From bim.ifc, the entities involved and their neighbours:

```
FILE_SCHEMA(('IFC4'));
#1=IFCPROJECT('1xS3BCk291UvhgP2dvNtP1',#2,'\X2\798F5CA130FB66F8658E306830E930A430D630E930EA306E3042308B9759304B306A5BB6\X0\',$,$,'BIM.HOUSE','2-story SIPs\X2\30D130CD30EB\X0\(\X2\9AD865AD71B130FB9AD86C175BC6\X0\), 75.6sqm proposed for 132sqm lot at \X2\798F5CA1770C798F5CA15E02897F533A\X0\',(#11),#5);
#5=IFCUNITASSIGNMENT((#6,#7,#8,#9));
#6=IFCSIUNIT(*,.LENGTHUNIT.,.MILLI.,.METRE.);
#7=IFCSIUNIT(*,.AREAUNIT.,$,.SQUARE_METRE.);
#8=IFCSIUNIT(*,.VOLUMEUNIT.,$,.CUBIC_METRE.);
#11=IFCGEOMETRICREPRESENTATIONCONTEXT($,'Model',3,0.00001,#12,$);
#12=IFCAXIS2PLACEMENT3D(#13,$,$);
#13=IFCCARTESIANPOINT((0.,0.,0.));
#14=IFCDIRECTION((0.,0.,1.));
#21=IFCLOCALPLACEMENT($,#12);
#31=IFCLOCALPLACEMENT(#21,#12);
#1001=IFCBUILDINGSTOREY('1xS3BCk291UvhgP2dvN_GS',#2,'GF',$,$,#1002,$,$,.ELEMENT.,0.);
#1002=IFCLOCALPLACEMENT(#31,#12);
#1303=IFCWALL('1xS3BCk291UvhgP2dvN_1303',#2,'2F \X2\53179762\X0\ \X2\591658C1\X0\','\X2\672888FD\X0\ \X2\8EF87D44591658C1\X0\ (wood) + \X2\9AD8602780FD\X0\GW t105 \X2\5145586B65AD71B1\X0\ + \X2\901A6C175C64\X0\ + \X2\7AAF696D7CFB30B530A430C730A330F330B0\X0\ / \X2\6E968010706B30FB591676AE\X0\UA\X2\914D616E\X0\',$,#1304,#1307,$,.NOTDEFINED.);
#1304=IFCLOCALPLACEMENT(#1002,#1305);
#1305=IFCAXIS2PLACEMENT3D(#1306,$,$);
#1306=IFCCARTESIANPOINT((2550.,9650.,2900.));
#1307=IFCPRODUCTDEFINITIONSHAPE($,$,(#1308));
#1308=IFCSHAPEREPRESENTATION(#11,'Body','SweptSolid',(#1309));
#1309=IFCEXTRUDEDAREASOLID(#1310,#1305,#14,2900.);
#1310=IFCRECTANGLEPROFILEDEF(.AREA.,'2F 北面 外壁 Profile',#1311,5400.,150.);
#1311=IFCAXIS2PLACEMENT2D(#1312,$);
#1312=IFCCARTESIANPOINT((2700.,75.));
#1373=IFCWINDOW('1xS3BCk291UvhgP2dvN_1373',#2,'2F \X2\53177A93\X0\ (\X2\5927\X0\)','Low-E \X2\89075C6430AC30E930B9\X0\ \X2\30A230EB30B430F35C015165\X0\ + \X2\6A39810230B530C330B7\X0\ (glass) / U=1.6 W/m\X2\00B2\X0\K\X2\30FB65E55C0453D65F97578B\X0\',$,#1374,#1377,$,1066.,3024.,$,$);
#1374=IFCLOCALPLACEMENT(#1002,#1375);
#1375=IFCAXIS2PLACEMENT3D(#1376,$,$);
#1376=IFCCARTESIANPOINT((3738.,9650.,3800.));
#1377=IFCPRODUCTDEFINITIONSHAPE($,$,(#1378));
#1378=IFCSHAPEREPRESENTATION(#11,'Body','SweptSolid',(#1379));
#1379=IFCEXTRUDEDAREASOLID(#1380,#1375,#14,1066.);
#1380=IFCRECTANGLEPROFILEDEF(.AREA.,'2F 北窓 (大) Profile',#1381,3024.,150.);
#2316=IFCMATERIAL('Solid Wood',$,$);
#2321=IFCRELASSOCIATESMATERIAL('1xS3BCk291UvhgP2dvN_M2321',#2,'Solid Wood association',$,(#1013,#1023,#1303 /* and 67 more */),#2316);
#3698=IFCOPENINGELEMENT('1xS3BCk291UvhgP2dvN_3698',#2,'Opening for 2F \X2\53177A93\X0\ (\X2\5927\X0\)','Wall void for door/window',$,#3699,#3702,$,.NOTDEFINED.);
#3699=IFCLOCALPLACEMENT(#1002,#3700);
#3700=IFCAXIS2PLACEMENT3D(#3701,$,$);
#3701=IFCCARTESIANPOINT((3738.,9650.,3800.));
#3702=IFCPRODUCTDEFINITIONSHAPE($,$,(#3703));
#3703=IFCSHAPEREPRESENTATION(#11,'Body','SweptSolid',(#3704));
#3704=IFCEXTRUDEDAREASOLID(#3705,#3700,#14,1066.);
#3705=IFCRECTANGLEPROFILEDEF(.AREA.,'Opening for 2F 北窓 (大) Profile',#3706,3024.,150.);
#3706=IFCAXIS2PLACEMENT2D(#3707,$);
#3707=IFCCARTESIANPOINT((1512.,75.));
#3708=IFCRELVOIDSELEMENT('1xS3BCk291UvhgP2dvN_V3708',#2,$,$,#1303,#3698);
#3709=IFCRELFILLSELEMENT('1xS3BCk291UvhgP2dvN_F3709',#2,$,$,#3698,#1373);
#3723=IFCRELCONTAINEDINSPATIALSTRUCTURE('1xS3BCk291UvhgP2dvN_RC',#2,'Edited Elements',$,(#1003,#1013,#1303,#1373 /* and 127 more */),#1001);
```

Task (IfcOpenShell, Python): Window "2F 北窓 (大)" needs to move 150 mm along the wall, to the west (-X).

```python
import ifcopenshell
import ifcopenshell.api.geometry
import ifcopenshell.util.placement
import ifcopenshell.util.unit

model = ifcopenshell.open("bim.ifc")
unit_scale = ifcopenshell.util.unit.calculate_unit_scale(model)

window = model.by_guid("1xS3BCk291UvhgP2dvN_1373")
opening = window.FillsVoids[0].RelatingOpeningElement
wall = opening.VoidsElements[0].RelatingBuildingElement

wall_matrix = ifcopenshell.util.placement.get_local_placement(wall.ObjectPlacement)
shift = wall_matrix[:3, 0] * -0.15 / unit_scale
before = ifcopenshell.util.placement.get_local_placement(window.ObjectPlacement)[:3, 3].copy()

# The window is not placed relative to its opening, so move both.
for product in (opening, window):
    matrix = ifcopenshell.util.placement.get_local_placement(product.ObjectPlacement)
    matrix[:3, 3] += shift
    ifcopenshell.api.geometry.edit_object_placement(model, product=product, matrix=matrix, is_si=False)

after = ifcopenshell.util.placement.get_local_placement(window.ObjectPlacement)[:3, 3]
print("window moved by", (after - before).round(3) + 0.0)

model.write("bim-out.ifc")
```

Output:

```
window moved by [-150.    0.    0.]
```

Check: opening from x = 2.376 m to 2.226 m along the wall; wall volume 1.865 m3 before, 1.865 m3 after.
